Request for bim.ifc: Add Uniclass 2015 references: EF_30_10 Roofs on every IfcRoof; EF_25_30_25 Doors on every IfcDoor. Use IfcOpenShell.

First a look at what the model holds.

```python
import ifcopenshell

model = ifcopenshell.open("bim.ifc")
print(model.schema)
print("classifications:", [c.Name for c in model.by_type("IfcClassification")])
for ifc_class in ("IfcDoor", "IfcRoof", "IfcStair", "IfcWall", "IfcWindow"):
    print(ifc_class, len(model.by_type(ifc_class)))
```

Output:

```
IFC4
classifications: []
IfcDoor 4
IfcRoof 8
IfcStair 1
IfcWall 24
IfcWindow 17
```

```python
import ifcopenshell
import ifcopenshell.api.classification

model = ifcopenshell.open("bim.ifc")

system = ifcopenshell.api.classification.add_classification(model, classification="Uniclass 2015")

codes = {
    "IfcRoof": ("EF_30_10", "Roofs"),
    "IfcDoor": ("EF_25_30_25", "Doors"),
}
for ifc_class, (code, name) in codes.items():
    products = model.by_type(ifc_class)
    ifcopenshell.api.classification.add_reference(
        model, products=products, classification=system, identification=code, name=name
    )
    print(code, len(products))

model.write("bim_v2.ifc")
```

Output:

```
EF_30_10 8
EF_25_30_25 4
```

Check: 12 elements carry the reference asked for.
